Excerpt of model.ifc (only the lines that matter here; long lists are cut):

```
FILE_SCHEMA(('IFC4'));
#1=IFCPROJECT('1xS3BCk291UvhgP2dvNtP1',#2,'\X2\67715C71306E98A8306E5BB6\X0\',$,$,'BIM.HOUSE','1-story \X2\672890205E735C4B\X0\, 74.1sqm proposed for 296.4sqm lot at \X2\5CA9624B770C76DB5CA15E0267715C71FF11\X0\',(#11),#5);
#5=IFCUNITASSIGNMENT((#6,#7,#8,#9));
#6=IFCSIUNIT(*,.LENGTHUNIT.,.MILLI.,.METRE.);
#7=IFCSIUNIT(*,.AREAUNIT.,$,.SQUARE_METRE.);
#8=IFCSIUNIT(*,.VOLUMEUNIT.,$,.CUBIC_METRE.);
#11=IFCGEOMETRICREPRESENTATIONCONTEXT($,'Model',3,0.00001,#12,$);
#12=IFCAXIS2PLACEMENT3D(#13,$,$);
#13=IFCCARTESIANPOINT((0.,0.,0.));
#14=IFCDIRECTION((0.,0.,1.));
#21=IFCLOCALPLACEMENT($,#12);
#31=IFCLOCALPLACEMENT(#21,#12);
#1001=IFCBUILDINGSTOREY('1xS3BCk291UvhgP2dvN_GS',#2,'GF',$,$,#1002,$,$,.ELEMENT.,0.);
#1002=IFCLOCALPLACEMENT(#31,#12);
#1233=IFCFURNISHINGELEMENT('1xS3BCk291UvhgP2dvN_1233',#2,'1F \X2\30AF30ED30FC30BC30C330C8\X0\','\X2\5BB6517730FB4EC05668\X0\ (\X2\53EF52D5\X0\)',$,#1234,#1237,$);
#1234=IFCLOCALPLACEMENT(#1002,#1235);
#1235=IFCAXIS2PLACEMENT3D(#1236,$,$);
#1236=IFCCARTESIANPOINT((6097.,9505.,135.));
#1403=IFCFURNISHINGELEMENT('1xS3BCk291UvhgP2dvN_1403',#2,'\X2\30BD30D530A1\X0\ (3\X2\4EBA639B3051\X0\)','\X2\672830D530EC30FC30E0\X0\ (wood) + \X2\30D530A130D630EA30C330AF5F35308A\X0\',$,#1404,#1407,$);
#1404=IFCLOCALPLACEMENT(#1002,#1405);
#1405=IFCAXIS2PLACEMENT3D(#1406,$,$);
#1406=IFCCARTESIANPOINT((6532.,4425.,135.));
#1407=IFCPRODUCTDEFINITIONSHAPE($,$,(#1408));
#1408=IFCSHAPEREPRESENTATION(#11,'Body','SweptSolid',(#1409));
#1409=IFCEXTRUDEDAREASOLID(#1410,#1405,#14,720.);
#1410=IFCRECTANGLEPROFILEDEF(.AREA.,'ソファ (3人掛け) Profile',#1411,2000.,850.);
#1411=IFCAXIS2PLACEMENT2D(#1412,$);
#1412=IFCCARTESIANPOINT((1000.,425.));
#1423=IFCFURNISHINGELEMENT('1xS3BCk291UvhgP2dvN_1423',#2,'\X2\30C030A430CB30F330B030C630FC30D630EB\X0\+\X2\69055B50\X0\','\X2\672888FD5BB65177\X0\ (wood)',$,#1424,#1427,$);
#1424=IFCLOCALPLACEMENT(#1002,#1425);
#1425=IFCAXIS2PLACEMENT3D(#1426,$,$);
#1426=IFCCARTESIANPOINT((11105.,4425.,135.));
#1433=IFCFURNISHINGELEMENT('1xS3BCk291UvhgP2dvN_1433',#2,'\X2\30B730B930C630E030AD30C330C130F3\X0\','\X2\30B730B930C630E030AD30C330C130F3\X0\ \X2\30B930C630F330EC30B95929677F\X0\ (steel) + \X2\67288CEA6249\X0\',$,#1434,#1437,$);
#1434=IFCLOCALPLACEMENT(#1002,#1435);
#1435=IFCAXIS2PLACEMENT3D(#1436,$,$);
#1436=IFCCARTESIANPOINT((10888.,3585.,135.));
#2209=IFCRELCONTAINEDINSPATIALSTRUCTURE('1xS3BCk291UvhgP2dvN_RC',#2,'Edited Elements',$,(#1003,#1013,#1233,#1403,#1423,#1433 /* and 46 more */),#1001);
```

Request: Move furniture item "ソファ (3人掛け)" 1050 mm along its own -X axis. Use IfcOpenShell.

```python
import ifcopenshell
import ifcopenshell.api.geometry
import ifcopenshell.util.placement
import ifcopenshell.util.unit

model = ifcopenshell.open("model.ifc")
unit_scale = ifcopenshell.util.unit.calculate_unit_scale(model)

item = model.by_guid("1xS3BCk291UvhgP2dvN_1403")
matrix = ifcopenshell.util.placement.get_local_placement(item.ObjectPlacement)
matrix[:3, 3] -= matrix[:3, 0] * 1.05 / unit_scale
ifcopenshell.api.geometry.edit_object_placement(model, product=item, matrix=matrix, is_si=False)

print(ifcopenshell.util.placement.get_local_placement(item.ObjectPlacement).round(3) + 0.0)

model.write("model-out.ifc")
```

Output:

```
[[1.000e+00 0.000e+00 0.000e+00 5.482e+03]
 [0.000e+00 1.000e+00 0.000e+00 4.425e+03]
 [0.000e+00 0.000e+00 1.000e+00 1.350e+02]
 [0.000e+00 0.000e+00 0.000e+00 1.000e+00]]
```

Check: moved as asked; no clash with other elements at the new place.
